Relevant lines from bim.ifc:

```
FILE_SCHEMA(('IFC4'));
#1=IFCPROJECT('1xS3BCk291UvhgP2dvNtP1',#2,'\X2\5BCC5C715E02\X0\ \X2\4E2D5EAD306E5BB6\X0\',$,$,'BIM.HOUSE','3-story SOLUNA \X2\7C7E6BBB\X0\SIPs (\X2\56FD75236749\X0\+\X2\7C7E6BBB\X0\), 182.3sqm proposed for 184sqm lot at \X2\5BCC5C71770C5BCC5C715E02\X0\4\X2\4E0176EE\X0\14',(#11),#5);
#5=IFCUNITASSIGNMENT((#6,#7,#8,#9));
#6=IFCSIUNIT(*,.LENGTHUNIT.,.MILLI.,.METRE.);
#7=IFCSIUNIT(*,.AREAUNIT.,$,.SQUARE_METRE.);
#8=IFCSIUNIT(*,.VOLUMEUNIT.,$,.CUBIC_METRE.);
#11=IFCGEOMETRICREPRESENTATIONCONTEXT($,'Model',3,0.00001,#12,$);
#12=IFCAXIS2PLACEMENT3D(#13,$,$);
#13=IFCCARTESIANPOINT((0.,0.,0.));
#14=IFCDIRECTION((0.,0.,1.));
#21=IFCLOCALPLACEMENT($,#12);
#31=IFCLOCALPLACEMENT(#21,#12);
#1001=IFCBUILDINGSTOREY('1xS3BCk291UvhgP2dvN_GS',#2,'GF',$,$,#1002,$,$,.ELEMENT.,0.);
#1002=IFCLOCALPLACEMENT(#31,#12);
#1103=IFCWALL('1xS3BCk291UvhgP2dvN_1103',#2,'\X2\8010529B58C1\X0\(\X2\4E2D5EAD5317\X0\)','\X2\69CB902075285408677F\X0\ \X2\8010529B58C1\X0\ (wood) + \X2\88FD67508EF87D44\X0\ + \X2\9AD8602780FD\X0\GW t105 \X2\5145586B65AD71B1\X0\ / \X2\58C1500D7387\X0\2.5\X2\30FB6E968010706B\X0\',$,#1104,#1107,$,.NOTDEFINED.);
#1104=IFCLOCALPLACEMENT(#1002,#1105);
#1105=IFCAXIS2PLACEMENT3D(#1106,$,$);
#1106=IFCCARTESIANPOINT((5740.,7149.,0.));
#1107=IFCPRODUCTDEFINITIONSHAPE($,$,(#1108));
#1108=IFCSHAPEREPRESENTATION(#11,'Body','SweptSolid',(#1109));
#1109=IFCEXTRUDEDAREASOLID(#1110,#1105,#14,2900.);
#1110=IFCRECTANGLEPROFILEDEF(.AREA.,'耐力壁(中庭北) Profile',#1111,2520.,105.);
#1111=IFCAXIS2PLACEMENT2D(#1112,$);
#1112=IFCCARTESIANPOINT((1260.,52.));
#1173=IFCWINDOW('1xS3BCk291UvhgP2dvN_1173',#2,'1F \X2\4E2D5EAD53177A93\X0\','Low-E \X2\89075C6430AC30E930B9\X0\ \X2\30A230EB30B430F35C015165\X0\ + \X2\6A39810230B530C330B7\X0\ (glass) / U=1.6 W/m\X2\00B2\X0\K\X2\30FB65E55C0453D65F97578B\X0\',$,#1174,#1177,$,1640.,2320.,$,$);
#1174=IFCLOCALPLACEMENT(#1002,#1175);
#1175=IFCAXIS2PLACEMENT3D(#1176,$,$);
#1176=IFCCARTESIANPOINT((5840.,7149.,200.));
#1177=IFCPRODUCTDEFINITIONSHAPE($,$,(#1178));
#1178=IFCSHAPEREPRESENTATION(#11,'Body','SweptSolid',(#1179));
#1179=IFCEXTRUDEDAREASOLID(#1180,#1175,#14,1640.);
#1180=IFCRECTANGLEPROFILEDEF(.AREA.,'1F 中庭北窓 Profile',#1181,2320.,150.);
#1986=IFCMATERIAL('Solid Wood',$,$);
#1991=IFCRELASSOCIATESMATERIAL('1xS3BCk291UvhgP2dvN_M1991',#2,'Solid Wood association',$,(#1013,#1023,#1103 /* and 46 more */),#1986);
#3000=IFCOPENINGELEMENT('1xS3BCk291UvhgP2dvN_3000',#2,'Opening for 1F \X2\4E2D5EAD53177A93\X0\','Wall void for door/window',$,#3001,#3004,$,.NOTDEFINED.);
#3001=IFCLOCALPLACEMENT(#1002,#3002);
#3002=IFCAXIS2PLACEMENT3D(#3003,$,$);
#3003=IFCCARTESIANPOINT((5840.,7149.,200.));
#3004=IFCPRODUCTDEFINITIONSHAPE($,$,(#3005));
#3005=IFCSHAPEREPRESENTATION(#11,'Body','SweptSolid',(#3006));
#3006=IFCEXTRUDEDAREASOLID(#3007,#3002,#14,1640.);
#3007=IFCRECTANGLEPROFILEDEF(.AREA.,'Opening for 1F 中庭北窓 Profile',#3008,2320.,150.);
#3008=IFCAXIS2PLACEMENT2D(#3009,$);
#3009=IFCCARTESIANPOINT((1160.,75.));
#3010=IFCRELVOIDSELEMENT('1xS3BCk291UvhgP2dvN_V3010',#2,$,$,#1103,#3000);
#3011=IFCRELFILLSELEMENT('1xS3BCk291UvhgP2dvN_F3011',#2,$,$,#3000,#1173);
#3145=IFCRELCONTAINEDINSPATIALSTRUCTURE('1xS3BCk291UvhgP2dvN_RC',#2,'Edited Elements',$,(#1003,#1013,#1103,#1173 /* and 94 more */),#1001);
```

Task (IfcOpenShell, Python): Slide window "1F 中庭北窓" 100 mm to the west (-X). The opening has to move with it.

```python
import ifcopenshell
import ifcopenshell.api.geometry
import ifcopenshell.util.placement
import ifcopenshell.util.unit

model = ifcopenshell.open("bim.ifc")
unit_scale = ifcopenshell.util.unit.calculate_unit_scale(model)

window = model.by_guid("1xS3BCk291UvhgP2dvN_1173")
opening = window.FillsVoids[0].RelatingOpeningElement
wall = opening.VoidsElements[0].RelatingBuildingElement

wall_matrix = ifcopenshell.util.placement.get_local_placement(wall.ObjectPlacement)
shift = wall_matrix[:3, 0] * -0.1 / unit_scale
before = ifcopenshell.util.placement.get_local_placement(window.ObjectPlacement)[:3, 3].copy()

# The window is not placed relative to its opening, so move both.
for product in (opening, window):
    matrix = ifcopenshell.util.placement.get_local_placement(product.ObjectPlacement)
    matrix[:3, 3] += shift
    ifcopenshell.api.geometry.edit_object_placement(model, product=product, matrix=matrix, is_si=False)

after = ifcopenshell.util.placement.get_local_placement(window.ObjectPlacement)[:3, 3]
print("window moved by", (after - before).round(3) + 0.0)

model.write("bim_updated.ifc")
```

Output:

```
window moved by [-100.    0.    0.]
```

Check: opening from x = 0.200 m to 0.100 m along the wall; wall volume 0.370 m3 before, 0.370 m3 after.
